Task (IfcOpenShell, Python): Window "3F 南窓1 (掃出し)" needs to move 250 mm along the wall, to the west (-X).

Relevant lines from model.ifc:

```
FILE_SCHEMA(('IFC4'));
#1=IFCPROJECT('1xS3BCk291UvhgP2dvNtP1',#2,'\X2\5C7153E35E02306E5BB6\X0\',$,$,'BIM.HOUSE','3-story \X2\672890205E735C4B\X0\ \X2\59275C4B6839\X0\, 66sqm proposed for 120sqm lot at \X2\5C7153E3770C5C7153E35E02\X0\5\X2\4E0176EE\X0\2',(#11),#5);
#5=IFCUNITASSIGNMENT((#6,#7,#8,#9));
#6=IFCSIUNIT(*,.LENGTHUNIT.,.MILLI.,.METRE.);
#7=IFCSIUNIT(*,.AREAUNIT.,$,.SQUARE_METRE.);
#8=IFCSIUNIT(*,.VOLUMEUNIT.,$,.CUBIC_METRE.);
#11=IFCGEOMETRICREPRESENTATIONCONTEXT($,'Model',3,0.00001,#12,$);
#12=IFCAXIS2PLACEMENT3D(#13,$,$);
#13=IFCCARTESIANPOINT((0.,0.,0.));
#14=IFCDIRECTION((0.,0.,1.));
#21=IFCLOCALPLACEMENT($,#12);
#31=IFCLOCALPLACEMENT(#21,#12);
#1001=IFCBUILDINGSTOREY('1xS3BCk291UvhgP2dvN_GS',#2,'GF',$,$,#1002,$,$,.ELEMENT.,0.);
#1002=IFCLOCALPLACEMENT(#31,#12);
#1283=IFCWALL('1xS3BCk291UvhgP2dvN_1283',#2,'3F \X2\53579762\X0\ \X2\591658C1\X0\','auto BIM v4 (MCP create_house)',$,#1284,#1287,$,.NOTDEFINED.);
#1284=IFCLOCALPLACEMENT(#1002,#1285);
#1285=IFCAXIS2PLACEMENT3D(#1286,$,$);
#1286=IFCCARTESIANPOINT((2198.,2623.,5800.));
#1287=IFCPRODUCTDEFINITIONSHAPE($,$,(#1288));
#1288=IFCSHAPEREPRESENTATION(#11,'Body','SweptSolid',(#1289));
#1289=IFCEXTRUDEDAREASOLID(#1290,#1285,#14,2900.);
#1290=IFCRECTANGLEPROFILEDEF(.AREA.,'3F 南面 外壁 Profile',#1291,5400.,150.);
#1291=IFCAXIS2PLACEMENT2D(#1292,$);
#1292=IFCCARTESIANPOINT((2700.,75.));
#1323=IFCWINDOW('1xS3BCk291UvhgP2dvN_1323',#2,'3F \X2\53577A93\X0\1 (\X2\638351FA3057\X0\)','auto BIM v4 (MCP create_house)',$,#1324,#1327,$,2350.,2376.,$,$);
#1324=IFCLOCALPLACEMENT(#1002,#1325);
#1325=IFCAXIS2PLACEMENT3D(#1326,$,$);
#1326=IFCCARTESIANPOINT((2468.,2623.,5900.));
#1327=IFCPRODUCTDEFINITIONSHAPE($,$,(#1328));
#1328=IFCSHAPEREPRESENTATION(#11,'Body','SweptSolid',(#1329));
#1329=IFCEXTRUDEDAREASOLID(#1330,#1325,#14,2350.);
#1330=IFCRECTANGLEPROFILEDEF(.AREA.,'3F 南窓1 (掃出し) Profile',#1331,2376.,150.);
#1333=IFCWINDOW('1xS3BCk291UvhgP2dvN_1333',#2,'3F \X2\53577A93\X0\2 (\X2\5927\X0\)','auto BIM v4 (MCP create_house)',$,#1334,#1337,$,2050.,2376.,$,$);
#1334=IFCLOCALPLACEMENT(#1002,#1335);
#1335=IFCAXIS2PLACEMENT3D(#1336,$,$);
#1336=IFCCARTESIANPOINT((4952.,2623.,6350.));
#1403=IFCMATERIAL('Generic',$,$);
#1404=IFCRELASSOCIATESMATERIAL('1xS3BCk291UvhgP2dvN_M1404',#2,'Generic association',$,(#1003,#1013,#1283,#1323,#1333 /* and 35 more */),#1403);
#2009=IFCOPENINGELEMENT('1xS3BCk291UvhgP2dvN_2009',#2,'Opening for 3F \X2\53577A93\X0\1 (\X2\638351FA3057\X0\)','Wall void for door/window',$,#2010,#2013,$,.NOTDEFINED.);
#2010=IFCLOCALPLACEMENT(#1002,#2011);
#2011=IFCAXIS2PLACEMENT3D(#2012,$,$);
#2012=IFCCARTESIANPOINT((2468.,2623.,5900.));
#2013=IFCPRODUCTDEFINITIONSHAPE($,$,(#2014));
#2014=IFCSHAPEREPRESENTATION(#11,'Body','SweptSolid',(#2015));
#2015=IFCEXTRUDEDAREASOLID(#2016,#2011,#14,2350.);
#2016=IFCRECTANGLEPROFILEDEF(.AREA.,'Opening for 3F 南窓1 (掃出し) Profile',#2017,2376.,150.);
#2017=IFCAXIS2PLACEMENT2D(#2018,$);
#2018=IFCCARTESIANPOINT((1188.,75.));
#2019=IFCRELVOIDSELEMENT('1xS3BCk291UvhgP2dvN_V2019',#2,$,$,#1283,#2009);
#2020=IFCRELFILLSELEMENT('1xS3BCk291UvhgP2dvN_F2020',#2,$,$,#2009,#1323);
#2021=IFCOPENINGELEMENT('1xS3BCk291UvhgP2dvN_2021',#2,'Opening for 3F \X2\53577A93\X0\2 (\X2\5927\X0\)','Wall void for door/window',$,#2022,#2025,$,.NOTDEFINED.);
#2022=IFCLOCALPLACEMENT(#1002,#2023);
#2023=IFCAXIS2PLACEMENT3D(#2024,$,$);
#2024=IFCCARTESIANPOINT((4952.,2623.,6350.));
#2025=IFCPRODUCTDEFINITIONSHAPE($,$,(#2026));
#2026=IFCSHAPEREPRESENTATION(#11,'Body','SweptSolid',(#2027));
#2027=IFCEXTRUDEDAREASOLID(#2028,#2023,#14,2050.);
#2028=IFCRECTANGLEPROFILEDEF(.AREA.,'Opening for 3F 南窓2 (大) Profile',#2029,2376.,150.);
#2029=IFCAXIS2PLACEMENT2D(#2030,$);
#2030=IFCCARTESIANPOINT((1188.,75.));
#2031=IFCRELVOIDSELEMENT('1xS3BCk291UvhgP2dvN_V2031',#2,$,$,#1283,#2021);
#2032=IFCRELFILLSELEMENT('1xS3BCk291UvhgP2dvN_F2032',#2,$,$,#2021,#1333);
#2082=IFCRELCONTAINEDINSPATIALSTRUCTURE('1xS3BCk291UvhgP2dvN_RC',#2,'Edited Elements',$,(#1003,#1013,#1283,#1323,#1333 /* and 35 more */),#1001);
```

```python
import ifcopenshell
import ifcopenshell.api.geometry
import ifcopenshell.util.placement

model = ifcopenshell.open("model.ifc")

window = model.by_id(1323)
opening = window.FillsVoids[0].RelatingOpeningElement
wall = opening.VoidsElements[0].RelatingBuildingElement

wall_matrix = ifcopenshell.util.placement.get_local_placement(wall.ObjectPlacement)
shift = wall_matrix[:3, 0] * -250.0
before = ifcopenshell.util.placement.get_local_placement(window.ObjectPlacement)[:3, 3].copy()

# The window is not placed relative to its opening, so move both.
for product in (opening, window):
    matrix = ifcopenshell.util.placement.get_local_placement(product.ObjectPlacement)
    matrix[:3, 3] += shift
    ifcopenshell.api.geometry.edit_object_placement(model, product=product, matrix=matrix, is_si=False)

after = ifcopenshell.util.placement.get_local_placement(window.ObjectPlacement)[:3, 3]
print("window moved by", (after - before).round(3) + 0.0)

model.write("model-out.ifc")
```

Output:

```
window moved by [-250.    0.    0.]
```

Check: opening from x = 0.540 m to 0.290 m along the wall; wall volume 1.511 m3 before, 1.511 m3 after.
